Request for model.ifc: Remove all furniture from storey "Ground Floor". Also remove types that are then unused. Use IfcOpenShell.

First a look at what the model holds.

```python
import ifcopenshell
import ifcopenshell.util.element

model = ifcopenshell.open("model.ifc")
print(model.schema)
storey = next(s for s in model.by_type("IfcBuildingStorey") if s.Name == "Ground Floor")
furniture = [e for e in ifcopenshell.util.element.get_decomposition(storey) if e.is_a("IfcFurnishingElement")]
seen = {}
for e in furniture:
    element_type = ifcopenshell.util.element.get_type(e)
    name = element_type.Name if element_type not in (None, e) else None
    seen[name] = seen.get(name, 0) + 1
for name, count in sorted(seen.items(), key=str):
    print(count, "x", name)
```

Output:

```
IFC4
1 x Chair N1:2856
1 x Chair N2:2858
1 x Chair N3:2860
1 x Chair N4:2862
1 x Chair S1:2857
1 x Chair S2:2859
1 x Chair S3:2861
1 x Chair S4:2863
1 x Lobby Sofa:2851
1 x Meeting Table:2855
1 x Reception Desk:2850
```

```python
import ifcopenshell
import ifcopenshell.api.root
import ifcopenshell.util.element

model = ifcopenshell.open("model.ifc")

storey = next(s for s in model.by_type("IfcBuildingStorey") if s.Name == "Ground Floor")
furniture = [e for e in ifcopenshell.util.element.get_decomposition(storey) if e.is_a("IfcFurnishingElement")]
types = {ifcopenshell.util.element.get_type(e) for e in furniture} - {None, *furniture}

for e in furniture:
    ifcopenshell.api.root.remove_product(model, product=e)
print(len(furniture), "removed")

unused = [t for t in types if not ifcopenshell.util.element.get_types(t)]
for t in unused:
    ifcopenshell.api.root.remove_product(model, product=t)
print(len(unused), "unused types removed")

model.write("model_updated.ifc")
```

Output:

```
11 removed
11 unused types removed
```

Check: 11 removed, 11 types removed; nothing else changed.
